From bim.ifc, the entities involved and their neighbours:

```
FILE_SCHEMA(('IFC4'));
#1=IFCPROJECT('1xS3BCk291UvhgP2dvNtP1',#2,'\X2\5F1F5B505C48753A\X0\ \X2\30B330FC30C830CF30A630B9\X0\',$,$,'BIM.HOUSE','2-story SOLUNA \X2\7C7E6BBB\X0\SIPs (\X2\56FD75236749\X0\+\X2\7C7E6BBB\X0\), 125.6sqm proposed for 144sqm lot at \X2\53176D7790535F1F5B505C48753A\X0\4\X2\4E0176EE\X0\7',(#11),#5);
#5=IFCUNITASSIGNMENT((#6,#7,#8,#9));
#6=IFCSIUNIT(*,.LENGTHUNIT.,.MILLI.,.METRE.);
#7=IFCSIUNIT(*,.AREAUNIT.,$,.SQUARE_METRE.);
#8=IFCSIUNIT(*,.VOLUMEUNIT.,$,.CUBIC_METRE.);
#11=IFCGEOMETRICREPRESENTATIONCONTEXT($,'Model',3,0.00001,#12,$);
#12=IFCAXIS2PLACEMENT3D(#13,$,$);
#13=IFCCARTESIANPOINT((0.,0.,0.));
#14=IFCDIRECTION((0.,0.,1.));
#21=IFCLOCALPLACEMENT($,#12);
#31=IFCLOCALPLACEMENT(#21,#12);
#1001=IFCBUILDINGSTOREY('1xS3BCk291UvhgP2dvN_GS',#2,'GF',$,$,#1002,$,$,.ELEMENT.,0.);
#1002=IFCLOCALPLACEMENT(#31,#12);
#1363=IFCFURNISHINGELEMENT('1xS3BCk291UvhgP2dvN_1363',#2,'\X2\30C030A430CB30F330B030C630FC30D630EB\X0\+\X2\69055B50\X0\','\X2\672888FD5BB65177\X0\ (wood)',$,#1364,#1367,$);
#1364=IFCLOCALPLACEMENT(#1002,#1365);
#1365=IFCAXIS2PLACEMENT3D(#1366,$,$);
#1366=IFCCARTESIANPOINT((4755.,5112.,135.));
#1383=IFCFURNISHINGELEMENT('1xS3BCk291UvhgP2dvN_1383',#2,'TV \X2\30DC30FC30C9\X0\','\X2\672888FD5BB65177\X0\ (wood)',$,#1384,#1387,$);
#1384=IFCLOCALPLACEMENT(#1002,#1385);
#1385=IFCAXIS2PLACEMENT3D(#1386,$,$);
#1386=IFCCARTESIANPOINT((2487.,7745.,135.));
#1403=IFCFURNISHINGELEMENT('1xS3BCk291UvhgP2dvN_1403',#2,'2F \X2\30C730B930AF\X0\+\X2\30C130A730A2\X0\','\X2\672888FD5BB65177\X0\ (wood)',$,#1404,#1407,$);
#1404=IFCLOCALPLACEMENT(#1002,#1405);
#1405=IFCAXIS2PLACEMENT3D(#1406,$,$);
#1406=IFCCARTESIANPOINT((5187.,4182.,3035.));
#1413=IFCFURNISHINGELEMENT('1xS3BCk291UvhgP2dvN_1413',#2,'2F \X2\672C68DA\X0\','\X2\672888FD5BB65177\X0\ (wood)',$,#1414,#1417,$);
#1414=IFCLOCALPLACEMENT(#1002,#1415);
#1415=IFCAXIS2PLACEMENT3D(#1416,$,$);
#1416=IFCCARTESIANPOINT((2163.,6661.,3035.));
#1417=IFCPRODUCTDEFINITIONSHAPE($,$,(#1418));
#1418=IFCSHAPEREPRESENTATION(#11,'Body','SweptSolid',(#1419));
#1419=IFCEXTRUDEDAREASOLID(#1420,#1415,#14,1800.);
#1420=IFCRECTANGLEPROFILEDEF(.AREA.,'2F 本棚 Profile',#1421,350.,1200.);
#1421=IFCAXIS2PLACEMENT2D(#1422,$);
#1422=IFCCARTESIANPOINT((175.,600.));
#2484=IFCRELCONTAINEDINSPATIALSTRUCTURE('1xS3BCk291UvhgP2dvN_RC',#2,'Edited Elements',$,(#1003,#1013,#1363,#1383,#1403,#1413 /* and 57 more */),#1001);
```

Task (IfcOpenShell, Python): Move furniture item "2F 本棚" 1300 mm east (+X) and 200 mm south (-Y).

```python
import ifcopenshell
import ifcopenshell.api.geometry
import ifcopenshell.util.placement
import ifcopenshell.util.unit

model = ifcopenshell.open("bim.ifc")
unit_scale = ifcopenshell.util.unit.calculate_unit_scale(model)

item = model.by_guid("1xS3BCk291UvhgP2dvN_1413")
matrix = ifcopenshell.util.placement.get_local_placement(item.ObjectPlacement)
matrix[0, 3] += 1.3 / unit_scale
matrix[1, 3] -= 0.2 / unit_scale
ifcopenshell.api.geometry.edit_object_placement(model, product=item, matrix=matrix, is_si=False)

print(ifcopenshell.util.placement.get_local_placement(item.ObjectPlacement).round(3) + 0.0)

model.write("bim_updated.ifc")
```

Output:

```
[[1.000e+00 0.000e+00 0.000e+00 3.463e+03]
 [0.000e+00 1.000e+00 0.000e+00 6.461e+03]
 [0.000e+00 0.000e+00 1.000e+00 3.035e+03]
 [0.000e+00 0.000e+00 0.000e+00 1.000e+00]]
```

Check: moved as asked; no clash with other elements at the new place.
